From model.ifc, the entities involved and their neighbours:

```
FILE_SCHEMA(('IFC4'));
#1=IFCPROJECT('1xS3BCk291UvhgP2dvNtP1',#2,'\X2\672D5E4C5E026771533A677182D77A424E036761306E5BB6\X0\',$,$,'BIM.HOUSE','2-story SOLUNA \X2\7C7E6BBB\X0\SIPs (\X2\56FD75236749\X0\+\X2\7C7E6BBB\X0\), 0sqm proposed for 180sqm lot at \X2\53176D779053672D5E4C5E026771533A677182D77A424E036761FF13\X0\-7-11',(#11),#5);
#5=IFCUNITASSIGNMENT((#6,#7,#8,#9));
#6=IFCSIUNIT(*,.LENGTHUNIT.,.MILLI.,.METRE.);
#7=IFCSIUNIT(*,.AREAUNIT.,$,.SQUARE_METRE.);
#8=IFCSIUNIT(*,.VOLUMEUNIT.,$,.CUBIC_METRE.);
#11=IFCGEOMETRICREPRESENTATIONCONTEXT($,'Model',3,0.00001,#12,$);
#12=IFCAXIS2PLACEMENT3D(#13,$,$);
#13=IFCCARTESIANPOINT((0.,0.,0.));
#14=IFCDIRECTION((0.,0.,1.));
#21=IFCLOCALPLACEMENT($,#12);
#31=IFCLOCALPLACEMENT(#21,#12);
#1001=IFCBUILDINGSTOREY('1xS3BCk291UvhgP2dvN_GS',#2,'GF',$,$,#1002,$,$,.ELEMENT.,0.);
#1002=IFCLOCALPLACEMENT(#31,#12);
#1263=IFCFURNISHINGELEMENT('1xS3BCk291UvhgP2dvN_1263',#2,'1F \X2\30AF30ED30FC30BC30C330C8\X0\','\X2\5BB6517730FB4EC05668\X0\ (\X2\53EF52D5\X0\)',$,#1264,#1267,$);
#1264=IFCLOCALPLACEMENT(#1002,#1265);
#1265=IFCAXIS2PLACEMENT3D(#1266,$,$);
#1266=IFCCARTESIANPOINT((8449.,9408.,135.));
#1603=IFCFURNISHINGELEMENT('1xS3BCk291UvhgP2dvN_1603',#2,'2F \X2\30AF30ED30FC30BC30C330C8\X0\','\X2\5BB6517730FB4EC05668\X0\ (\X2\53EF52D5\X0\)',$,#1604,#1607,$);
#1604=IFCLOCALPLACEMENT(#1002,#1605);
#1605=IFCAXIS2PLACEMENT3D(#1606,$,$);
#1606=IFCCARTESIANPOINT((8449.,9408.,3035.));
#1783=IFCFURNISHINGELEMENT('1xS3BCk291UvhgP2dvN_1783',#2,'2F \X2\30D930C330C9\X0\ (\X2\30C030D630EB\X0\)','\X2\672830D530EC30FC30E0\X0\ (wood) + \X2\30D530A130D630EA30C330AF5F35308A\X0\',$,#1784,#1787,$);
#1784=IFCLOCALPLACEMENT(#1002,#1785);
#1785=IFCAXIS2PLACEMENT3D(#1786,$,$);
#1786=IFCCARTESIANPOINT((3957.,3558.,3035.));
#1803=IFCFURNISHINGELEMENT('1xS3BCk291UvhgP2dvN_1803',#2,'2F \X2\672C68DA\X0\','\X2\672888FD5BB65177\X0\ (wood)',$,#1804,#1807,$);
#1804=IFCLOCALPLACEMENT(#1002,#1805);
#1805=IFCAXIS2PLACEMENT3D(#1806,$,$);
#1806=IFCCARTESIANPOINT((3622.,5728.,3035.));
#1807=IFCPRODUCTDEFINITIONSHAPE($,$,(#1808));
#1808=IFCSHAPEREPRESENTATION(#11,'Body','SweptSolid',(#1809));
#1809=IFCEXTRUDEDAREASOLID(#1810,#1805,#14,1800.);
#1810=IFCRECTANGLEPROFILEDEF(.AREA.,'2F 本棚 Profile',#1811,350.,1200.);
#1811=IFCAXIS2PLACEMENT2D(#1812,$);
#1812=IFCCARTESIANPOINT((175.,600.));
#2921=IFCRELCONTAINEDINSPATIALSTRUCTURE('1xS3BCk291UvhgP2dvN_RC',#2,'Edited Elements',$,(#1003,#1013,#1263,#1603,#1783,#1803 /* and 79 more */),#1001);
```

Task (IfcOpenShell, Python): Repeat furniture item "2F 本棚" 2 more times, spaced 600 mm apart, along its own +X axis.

```python
import ifcopenshell
import ifcopenshell.api.geometry
import ifcopenshell.api.root
import ifcopenshell.util.element
import ifcopenshell.util.placement
import ifcopenshell.util.unit

model = ifcopenshell.open("model.ifc")
unit_scale = ifcopenshell.util.unit.calculate_unit_scale(model)


def reuse_history(source, copy):
    """copy_class also copies each property set's owner history, people and application; keep the originals."""
    for rel in copy.IsDefinedBy:
        if rel.is_a("IfcRelDefinesByProperties") and (history := rel.RelatingPropertyDefinition.OwnerHistory):
            rel.RelatingPropertyDefinition.OwnerHistory = source.OwnerHistory
            ifcopenshell.util.element.remove_deep2(model, history)


source = model.by_guid("1xS3BCk291UvhgP2dvN_1803")
base = ifcopenshell.util.placement.get_local_placement(source.ObjectPlacement)
step = base[:3, 0] * 0.6 / unit_scale

for i in range(1, 3):
    copy = ifcopenshell.api.root.copy_class(model, product=source)
    copy.Representation = ifcopenshell.util.element.copy_deep(
        model, source.Representation, exclude=["IfcGeometricRepresentationContext", "IfcRepresentationMap"]
    )
    reuse_history(source, copy)
    matrix = base.copy()
    matrix[:3, 3] += i * step
    print("added at", matrix[:3, 3].round(3) + 0.0)
    ifcopenshell.api.geometry.edit_object_placement(model, product=copy, matrix=matrix, is_si=False)

model.write("model_rev.ifc")
```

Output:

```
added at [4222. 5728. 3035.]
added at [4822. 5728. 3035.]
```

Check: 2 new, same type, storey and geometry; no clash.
